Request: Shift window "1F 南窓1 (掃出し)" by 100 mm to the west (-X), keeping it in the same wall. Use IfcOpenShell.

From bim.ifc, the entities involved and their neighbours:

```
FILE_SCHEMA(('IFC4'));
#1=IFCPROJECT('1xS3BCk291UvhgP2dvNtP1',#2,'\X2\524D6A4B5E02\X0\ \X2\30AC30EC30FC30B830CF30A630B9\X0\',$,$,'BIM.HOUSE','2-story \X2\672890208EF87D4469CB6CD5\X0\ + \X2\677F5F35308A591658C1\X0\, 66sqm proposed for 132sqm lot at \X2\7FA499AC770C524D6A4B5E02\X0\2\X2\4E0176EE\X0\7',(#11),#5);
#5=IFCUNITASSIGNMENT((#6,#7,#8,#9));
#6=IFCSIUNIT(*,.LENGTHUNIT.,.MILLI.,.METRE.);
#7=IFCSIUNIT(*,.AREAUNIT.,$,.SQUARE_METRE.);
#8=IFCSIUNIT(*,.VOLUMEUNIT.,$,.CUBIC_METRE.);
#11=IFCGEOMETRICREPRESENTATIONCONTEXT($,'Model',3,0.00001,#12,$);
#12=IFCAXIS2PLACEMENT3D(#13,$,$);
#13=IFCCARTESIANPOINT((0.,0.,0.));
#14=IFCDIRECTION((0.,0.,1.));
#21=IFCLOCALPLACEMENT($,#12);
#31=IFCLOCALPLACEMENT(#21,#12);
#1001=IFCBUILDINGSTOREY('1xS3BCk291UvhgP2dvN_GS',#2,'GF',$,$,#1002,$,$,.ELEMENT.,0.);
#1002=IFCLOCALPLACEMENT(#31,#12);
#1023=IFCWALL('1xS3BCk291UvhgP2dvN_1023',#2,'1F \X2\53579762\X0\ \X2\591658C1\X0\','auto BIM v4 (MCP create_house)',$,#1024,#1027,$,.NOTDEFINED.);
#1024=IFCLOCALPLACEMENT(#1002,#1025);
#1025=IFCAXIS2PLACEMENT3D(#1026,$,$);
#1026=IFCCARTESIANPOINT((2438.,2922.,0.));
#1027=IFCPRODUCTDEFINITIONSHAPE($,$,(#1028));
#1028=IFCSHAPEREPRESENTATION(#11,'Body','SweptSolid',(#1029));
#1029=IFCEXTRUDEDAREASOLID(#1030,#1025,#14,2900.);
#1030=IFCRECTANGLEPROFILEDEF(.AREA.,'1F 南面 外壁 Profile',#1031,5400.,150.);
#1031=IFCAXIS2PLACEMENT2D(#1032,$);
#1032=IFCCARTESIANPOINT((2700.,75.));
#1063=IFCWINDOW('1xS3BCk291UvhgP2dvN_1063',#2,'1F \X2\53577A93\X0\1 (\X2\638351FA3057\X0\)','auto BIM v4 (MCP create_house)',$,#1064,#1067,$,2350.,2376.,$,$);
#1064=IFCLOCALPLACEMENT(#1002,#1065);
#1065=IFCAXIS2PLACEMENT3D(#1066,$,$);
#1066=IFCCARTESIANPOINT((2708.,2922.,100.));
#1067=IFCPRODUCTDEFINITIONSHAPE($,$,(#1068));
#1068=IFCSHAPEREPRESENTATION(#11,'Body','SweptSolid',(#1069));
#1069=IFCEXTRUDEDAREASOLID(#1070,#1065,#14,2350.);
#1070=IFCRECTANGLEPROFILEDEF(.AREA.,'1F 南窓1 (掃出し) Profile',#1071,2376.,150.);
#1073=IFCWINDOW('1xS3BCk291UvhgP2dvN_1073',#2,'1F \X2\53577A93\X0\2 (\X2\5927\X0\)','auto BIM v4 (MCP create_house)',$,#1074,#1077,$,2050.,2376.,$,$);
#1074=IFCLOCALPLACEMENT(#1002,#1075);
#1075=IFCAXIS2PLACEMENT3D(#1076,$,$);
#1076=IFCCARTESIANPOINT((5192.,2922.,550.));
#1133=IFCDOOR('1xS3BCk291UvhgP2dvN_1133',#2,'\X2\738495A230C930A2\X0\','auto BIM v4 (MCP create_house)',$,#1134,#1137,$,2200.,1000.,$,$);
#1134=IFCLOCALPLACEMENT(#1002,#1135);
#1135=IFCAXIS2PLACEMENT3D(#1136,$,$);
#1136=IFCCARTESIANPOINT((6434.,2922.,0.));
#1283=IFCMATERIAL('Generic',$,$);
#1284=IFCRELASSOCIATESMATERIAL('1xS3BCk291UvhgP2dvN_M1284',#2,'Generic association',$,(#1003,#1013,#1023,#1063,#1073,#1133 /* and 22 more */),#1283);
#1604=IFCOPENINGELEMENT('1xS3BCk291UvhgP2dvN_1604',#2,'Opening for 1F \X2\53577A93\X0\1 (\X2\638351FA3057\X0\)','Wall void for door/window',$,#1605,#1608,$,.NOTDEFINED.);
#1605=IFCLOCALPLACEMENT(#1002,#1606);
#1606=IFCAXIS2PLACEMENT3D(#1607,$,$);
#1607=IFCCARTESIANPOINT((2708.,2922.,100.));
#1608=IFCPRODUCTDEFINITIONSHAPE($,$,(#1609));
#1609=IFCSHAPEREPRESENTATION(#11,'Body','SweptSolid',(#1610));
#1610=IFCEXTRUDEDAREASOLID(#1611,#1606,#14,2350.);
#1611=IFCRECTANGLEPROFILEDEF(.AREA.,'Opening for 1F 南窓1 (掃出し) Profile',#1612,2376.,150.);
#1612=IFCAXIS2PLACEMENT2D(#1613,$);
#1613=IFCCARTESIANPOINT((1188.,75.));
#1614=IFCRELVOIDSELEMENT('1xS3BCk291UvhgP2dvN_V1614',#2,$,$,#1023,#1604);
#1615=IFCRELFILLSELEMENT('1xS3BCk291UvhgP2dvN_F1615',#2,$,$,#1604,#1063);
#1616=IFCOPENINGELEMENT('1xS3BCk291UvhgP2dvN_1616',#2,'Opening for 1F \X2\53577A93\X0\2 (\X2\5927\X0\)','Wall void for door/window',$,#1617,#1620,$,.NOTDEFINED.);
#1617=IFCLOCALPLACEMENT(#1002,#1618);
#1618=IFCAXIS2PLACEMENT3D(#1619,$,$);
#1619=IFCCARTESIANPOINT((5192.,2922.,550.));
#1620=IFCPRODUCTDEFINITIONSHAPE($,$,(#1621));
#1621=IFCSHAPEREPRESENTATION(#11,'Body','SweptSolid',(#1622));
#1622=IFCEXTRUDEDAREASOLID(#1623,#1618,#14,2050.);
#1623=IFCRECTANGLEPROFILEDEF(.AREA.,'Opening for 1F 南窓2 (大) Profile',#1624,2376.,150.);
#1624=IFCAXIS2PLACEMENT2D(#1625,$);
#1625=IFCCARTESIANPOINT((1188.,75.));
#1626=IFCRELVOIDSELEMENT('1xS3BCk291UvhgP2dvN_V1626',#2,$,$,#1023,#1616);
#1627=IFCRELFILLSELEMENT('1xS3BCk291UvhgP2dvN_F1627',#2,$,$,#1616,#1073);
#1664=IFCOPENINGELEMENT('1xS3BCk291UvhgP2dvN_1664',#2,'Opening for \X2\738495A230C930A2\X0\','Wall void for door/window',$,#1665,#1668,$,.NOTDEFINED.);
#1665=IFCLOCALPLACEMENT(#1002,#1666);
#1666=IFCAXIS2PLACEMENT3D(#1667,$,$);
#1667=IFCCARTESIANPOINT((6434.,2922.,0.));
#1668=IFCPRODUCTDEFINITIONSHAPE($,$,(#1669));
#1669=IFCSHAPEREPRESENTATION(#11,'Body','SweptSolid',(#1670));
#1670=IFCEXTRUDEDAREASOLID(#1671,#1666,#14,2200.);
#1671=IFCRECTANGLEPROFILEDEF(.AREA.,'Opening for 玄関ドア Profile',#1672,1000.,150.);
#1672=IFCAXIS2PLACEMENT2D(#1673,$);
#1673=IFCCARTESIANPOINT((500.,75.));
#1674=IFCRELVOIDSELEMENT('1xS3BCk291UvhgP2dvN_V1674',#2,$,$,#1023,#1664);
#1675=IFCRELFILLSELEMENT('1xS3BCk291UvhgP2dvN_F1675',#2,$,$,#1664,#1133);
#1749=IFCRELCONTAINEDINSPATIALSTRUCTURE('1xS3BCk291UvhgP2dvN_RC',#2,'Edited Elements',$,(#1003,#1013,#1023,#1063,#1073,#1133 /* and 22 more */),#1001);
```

```python
import ifcopenshell
import ifcopenshell.api.geometry
import ifcopenshell.util.placement

model = ifcopenshell.open("bim.ifc")

window = model.by_guid("1xS3BCk291UvhgP2dvN_1063")
opening = window.FillsVoids[0].RelatingOpeningElement
wall = opening.VoidsElements[0].RelatingBuildingElement

wall_matrix = ifcopenshell.util.placement.get_local_placement(wall.ObjectPlacement)
shift = wall_matrix[:3, 0] * -100.0
before = ifcopenshell.util.placement.get_local_placement(window.ObjectPlacement)[:3, 3].copy()

# The window is not placed relative to its opening, so move both.
for product in (opening, window):
    matrix = ifcopenshell.util.placement.get_local_placement(product.ObjectPlacement)
    matrix[:3, 3] += shift
    ifcopenshell.api.geometry.edit_object_placement(model, product=product, matrix=matrix, is_si=False)

after = ifcopenshell.util.placement.get_local_placement(window.ObjectPlacement)[:3, 3]
print("window moved by", (after - before).round(3) + 0.0)

model.write("bim_rev.ifc")
```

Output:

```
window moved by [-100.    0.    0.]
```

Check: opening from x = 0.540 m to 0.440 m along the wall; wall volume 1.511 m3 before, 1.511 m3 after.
